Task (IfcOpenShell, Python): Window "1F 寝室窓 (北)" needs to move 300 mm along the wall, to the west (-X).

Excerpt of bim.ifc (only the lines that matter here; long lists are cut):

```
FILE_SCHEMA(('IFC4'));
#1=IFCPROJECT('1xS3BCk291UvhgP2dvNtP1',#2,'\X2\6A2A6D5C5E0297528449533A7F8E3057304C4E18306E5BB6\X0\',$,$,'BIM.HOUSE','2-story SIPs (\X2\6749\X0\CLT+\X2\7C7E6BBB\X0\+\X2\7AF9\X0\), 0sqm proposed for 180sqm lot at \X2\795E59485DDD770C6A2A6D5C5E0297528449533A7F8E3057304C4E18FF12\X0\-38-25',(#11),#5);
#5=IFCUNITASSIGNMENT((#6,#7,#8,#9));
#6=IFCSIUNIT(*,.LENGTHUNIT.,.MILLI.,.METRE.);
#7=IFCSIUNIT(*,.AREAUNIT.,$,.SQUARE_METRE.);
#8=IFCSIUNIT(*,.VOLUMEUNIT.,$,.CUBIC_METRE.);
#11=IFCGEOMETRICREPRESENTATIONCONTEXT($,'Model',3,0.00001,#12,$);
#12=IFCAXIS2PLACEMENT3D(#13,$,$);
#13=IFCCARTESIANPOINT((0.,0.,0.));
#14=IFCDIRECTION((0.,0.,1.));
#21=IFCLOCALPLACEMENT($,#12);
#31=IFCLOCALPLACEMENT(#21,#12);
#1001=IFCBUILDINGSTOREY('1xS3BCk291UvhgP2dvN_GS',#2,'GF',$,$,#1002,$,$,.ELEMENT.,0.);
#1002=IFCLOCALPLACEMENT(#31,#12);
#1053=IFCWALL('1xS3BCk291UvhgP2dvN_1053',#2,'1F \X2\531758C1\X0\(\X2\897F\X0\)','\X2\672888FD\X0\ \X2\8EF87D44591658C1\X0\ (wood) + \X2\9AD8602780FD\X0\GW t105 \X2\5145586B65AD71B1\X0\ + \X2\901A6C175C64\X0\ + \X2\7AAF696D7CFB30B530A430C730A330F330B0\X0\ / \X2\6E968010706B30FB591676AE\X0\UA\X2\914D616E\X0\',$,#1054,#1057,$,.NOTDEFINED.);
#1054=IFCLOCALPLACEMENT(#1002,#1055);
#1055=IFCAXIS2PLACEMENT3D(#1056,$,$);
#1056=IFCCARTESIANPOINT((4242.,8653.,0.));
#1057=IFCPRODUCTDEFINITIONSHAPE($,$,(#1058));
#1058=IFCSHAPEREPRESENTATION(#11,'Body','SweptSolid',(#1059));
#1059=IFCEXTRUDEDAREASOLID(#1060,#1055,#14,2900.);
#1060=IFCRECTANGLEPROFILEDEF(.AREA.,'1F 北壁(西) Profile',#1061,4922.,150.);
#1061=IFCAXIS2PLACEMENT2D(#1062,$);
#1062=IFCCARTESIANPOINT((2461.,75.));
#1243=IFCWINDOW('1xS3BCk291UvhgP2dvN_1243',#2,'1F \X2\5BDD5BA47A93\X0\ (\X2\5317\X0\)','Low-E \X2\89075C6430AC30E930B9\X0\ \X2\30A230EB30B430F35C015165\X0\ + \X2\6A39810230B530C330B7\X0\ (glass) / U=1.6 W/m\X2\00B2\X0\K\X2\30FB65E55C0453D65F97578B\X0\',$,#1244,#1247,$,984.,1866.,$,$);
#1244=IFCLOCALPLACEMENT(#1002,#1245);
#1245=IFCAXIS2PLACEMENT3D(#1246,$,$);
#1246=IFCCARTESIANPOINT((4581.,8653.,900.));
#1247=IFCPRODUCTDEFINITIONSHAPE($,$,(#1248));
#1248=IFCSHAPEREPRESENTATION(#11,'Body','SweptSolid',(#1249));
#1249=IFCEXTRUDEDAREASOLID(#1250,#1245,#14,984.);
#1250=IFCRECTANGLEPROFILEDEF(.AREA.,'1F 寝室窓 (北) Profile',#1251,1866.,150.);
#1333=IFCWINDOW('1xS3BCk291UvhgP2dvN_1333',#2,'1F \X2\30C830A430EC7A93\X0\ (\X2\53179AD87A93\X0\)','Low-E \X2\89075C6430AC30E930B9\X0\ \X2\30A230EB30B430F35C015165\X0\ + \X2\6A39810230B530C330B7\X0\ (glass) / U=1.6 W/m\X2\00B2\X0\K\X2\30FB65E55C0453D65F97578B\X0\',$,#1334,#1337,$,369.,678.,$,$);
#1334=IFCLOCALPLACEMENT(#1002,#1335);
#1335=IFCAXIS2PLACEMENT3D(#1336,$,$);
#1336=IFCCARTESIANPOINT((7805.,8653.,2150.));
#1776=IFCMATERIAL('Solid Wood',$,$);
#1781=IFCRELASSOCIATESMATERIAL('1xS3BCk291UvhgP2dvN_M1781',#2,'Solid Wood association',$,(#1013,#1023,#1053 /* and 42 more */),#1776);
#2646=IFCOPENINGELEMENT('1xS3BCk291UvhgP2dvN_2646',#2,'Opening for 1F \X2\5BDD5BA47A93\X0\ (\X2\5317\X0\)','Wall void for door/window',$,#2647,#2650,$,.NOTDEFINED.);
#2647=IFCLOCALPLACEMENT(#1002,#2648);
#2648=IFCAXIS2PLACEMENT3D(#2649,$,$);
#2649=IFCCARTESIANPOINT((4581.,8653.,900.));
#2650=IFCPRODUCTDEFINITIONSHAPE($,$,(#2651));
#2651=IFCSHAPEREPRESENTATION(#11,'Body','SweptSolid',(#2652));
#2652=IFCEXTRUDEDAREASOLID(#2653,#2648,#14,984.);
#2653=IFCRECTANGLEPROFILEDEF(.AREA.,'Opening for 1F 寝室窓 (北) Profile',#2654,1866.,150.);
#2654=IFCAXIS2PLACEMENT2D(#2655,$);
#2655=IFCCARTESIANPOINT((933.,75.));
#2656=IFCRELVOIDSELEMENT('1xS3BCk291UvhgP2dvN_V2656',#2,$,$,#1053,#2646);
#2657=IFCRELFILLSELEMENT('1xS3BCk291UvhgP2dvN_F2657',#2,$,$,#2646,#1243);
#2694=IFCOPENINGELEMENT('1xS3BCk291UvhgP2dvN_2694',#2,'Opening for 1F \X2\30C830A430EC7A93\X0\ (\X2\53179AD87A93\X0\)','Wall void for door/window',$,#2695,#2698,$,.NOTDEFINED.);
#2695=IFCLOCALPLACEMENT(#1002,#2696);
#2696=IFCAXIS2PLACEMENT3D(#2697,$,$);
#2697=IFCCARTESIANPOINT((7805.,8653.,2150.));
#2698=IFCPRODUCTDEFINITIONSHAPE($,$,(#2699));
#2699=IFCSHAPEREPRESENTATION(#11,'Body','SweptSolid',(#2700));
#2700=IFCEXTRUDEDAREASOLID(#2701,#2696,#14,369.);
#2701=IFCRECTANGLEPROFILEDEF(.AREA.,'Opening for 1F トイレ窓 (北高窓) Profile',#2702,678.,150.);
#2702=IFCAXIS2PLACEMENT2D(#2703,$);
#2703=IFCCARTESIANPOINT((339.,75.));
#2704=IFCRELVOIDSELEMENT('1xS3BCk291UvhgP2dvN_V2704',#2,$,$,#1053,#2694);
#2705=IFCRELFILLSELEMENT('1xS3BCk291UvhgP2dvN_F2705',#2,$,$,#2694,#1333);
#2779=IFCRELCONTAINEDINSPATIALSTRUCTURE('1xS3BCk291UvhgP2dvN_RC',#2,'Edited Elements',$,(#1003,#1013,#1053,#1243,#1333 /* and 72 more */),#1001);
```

```python
import ifcopenshell
import ifcopenshell.api.geometry
import ifcopenshell.util.placement

model = ifcopenshell.open("bim.ifc")

window = model.by_guid("1xS3BCk291UvhgP2dvN_1243")
opening = window.FillsVoids[0].RelatingOpeningElement
wall = opening.VoidsElements[0].RelatingBuildingElement

wall_matrix = ifcopenshell.util.placement.get_local_placement(wall.ObjectPlacement)
shift = wall_matrix[:3, 0] * -300.0
before = ifcopenshell.util.placement.get_local_placement(window.ObjectPlacement)[:3, 3].copy()

# The window is not placed relative to its opening, so move both.
for product in (opening, window):
    matrix = ifcopenshell.util.placement.get_local_placement(product.ObjectPlacement)
    matrix[:3, 3] += shift
    ifcopenshell.api.geometry.edit_object_placement(model, product=product, matrix=matrix, is_si=False)

after = ifcopenshell.util.placement.get_local_placement(window.ObjectPlacement)[:3, 3]
print("window moved by", (after - before).round(3) + 0.0)

model.write("bim-out.ifc")
```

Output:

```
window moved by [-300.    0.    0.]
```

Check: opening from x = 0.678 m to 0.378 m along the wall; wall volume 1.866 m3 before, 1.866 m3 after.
